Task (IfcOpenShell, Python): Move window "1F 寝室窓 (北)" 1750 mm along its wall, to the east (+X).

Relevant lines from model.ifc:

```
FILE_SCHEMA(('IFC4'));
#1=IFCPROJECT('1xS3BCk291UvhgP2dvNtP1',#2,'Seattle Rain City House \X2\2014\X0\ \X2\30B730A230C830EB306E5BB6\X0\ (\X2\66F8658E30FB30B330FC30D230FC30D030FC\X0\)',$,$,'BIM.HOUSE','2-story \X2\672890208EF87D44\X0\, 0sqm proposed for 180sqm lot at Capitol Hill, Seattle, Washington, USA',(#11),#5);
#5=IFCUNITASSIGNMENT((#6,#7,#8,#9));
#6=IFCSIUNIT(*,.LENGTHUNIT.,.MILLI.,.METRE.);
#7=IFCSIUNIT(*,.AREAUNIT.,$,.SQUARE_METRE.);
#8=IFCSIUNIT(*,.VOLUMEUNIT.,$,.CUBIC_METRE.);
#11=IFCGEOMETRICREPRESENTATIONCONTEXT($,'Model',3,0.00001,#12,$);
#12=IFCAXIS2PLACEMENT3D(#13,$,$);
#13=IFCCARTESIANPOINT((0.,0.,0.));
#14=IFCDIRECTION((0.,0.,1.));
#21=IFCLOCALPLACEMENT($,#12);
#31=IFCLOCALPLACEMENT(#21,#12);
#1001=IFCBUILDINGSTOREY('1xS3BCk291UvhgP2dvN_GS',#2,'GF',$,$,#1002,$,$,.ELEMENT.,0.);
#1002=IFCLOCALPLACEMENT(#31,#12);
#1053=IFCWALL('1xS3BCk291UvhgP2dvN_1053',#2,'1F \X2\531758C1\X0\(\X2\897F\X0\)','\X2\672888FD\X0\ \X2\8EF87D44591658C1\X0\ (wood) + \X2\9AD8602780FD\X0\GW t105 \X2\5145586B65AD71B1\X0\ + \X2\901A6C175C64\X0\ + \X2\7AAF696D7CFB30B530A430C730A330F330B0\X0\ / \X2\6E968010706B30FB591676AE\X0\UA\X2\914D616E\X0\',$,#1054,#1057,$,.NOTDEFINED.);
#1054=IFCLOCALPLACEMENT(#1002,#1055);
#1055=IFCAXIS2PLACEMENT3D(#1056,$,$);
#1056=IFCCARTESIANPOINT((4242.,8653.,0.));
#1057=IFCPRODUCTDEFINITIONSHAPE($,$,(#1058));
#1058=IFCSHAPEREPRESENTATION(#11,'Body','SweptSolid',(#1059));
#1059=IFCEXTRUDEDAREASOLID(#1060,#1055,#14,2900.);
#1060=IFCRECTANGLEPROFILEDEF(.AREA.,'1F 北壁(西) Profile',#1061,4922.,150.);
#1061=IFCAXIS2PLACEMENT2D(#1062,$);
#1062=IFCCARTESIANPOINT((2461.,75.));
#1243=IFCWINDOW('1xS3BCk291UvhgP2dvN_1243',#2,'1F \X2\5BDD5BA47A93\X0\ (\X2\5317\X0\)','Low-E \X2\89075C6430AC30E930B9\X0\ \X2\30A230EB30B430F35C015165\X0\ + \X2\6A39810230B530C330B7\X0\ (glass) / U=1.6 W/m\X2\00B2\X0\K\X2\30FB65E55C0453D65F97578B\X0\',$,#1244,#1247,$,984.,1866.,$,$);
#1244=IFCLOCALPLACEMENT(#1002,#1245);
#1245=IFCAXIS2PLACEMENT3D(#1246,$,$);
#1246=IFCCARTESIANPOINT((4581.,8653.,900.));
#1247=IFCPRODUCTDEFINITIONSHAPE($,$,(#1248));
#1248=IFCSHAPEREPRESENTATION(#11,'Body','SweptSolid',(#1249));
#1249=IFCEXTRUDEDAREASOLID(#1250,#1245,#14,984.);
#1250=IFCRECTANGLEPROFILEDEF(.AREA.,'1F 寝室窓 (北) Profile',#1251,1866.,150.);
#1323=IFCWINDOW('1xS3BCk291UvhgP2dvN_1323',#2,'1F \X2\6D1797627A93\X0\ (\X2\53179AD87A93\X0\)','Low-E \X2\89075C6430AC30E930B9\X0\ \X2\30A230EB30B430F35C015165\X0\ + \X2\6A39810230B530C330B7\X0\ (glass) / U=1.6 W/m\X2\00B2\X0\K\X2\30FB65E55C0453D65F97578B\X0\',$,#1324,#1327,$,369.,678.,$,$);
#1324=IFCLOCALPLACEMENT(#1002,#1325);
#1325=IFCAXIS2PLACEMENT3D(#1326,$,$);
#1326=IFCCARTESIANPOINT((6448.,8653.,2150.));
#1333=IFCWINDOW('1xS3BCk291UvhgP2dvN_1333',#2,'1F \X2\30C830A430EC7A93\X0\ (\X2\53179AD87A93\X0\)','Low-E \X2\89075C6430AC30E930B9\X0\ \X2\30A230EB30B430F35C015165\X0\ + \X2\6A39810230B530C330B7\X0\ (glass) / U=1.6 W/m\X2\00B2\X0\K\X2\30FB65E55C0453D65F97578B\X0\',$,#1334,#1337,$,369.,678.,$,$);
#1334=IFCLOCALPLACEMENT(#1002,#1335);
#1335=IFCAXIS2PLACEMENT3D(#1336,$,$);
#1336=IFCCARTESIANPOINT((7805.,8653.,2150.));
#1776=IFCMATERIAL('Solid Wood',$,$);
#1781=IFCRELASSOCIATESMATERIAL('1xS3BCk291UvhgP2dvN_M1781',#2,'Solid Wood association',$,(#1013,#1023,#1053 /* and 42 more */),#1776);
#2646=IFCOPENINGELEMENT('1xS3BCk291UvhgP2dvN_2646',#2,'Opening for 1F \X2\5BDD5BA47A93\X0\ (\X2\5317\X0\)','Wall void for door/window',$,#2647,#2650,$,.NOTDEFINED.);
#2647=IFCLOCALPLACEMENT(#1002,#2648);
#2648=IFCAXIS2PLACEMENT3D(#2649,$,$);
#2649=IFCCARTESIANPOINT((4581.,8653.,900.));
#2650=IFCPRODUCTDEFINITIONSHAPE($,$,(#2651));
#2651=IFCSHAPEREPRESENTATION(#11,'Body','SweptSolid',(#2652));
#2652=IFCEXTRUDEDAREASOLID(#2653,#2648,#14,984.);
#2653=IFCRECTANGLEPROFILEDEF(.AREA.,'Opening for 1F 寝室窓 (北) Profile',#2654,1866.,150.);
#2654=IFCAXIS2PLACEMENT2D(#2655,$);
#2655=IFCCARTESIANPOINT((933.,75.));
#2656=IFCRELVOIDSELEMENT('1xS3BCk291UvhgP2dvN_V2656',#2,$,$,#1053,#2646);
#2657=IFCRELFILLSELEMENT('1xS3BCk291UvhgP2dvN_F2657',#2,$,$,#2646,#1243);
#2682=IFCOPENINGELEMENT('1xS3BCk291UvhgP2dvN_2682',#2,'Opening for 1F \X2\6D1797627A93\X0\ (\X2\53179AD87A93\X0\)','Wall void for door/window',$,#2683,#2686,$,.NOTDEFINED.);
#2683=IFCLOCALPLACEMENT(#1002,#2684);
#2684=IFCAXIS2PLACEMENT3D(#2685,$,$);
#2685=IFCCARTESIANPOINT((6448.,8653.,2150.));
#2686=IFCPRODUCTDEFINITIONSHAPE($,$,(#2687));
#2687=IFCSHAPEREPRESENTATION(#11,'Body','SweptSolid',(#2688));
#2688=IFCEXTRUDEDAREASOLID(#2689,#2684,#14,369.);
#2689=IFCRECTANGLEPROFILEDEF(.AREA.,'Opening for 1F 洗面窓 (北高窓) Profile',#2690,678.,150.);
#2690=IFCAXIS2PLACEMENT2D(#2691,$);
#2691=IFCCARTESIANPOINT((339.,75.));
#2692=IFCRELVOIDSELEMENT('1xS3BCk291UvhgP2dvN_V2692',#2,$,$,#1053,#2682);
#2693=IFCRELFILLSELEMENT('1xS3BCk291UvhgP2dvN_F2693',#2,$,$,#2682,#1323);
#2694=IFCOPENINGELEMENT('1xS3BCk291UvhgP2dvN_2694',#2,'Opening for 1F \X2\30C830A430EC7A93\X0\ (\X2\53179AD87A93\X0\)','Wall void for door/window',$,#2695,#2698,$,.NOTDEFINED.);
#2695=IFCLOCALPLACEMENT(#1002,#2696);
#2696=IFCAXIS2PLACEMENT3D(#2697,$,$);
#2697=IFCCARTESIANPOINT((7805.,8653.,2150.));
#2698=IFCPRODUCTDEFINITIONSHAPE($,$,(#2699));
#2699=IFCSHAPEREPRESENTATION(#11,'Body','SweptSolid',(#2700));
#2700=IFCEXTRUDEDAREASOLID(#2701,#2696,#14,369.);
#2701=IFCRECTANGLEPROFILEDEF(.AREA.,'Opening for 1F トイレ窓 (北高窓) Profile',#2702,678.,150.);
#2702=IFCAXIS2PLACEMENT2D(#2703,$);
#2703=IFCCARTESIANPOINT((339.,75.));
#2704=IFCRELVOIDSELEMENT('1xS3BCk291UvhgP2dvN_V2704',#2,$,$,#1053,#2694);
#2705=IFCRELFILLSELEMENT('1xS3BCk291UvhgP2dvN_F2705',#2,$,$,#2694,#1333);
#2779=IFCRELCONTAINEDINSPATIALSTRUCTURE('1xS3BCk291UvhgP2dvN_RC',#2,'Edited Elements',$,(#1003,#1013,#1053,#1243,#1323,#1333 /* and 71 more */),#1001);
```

```python
import ifcopenshell
import ifcopenshell.api.geometry
import ifcopenshell.util.placement

model = ifcopenshell.open("model.ifc")

window = model.by_guid("1xS3BCk291UvhgP2dvN_1243")
opening = window.FillsVoids[0].RelatingOpeningElement
wall = opening.VoidsElements[0].RelatingBuildingElement

wall_matrix = ifcopenshell.util.placement.get_local_placement(wall.ObjectPlacement)
shift = wall_matrix[:3, 0] * 1750.0
before = ifcopenshell.util.placement.get_local_placement(window.ObjectPlacement)[:3, 3].copy()

# The window is not placed relative to its opening, so move both.
for product in (opening, window):
    matrix = ifcopenshell.util.placement.get_local_placement(product.ObjectPlacement)
    matrix[:3, 3] += shift
    ifcopenshell.api.geometry.edit_object_placement(model, product=product, matrix=matrix, is_si=False)

after = ifcopenshell.util.placement.get_local_placement(window.ObjectPlacement)[:3, 3]
print("window moved by", (after - before).round(3) + 0.0)

model.write("model-out.ifc")
```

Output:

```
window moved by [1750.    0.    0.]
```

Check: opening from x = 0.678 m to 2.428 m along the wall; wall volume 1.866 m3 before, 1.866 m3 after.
